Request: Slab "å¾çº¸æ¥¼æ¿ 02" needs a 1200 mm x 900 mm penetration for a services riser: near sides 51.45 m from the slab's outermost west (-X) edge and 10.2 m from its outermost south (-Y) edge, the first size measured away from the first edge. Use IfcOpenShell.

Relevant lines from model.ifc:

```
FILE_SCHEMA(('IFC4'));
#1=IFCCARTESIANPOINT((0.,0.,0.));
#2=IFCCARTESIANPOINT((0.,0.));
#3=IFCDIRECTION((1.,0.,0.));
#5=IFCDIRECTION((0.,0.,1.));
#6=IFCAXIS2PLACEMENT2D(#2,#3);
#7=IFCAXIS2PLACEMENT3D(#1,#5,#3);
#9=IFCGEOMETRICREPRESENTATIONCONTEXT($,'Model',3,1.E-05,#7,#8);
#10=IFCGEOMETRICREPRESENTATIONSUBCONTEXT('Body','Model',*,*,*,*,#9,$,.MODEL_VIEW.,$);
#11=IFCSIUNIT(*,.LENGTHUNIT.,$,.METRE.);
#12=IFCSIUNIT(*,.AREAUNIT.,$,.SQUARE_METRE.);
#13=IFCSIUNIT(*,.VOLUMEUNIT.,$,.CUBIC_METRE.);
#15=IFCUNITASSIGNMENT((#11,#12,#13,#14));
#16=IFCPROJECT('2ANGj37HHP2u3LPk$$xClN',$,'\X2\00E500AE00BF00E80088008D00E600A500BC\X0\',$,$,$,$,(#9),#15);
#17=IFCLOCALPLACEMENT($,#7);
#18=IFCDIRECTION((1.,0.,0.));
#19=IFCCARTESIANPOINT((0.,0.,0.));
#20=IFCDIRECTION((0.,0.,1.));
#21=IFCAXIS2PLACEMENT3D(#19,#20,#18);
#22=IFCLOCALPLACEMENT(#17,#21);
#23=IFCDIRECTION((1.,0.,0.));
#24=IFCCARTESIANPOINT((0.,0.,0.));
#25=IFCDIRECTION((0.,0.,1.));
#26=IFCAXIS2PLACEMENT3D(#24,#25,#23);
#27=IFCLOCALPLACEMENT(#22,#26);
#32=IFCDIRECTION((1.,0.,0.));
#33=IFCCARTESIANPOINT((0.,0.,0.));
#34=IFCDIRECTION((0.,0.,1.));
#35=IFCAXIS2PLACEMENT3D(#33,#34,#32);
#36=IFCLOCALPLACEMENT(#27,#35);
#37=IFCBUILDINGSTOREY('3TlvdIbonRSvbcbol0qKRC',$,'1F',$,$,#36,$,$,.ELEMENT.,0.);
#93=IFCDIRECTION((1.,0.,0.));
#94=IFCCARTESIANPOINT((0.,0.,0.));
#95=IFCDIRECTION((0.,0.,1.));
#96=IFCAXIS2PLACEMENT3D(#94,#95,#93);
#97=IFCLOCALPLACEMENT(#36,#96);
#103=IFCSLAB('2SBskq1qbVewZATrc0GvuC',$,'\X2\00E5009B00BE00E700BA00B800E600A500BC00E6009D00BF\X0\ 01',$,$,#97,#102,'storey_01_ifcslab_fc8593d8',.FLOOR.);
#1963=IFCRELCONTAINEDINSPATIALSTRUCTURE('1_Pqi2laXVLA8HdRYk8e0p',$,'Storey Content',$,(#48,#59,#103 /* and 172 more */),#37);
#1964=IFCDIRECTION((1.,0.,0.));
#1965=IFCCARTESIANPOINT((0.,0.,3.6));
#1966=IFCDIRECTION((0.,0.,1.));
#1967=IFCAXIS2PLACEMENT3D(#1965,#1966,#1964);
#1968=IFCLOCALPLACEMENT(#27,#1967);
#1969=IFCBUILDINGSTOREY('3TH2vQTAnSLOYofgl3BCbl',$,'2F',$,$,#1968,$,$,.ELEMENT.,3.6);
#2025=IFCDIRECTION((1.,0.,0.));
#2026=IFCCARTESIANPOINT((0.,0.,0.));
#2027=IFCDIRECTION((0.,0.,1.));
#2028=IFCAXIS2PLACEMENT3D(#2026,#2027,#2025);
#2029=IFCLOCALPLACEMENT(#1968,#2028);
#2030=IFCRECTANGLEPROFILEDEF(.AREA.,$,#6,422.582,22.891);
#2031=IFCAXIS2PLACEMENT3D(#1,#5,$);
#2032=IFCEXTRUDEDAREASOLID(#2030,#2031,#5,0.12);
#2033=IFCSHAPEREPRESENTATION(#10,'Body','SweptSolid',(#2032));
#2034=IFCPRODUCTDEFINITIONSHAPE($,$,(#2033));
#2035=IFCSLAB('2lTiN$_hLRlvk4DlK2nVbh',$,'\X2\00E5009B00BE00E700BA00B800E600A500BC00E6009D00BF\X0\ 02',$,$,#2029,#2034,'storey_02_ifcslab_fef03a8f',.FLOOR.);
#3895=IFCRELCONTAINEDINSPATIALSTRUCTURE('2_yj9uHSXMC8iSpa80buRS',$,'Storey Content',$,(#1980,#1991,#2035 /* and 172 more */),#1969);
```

```python
import numpy as np
import ifcopenshell
import ifcopenshell.api.feature
import ifcopenshell.api.geometry
import ifcopenshell.api.root
import ifcopenshell.geom
import ifcopenshell.util.placement
import ifcopenshell.util.representation
import ifcopenshell.util.shape
import ifcopenshell.util.unit

model = ifcopenshell.open("model.ifc")
unit_scale = ifcopenshell.util.unit.calculate_unit_scale(model)
settings = ifcopenshell.geom.settings()


def volume(element):
    """Net volume in cubic metres, openings subtracted."""
    shape = ifcopenshell.geom.create_shape(settings, element)
    return ifcopenshell.util.shape.get_volume(shape.geometry)


slab = model.by_id(2035)
before = volume(slab)

# Extent in the slab's own axes, in metres. The edges named are its -X and -Y sides.
slab_shape = ifcopenshell.geom.create_shape(settings, slab)
vertices = ifcopenshell.util.shape.get_vertices(slab_shape.geometry)
x_min, y_min, bottom = vertices.min(axis=0)
top = vertices[:, 2].max()

opening = ifcopenshell.api.root.create_entity(model, ifc_class="IfcOpeningElement", name="Services riser opening", predefined_type="OPENING")
context = ifcopenshell.util.representation.get_context(model, "Model", "Body", "MODEL_VIEW")
width, depth = 1.2, 0.9
outline = [(0.0, 0.0), (width, 0.0), (width, depth), (0.0, depth), (0.0, 0.0)]
# Overshoot both faces by 50 mm so the cut is clean.
shape = ifcopenshell.api.geometry.add_slab_representation(
    model, context=context, depth=top - bottom + 0.1, polyline=outline
)
ifcopenshell.api.geometry.assign_representation(model, product=opening, representation=shape)

matrix = ifcopenshell.util.placement.get_local_placement(slab.ObjectPlacement)
matrix[:, 3] = matrix @ np.append(np.array([x_min + 51.45, y_min + 10.2, bottom - 0.05]) / unit_scale, 1.0)
ifcopenshell.api.geometry.edit_object_placement(model, product=opening, matrix=matrix, is_si=False)
ifcopenshell.api.feature.add_feature(model, feature=opening, element=slab)

after = volume(slab)

print(f"slab volume {before:.3f} -> {after:.3f} m3")

model.write("model_edited.ifc")
```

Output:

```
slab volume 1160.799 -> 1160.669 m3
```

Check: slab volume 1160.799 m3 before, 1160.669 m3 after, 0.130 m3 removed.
